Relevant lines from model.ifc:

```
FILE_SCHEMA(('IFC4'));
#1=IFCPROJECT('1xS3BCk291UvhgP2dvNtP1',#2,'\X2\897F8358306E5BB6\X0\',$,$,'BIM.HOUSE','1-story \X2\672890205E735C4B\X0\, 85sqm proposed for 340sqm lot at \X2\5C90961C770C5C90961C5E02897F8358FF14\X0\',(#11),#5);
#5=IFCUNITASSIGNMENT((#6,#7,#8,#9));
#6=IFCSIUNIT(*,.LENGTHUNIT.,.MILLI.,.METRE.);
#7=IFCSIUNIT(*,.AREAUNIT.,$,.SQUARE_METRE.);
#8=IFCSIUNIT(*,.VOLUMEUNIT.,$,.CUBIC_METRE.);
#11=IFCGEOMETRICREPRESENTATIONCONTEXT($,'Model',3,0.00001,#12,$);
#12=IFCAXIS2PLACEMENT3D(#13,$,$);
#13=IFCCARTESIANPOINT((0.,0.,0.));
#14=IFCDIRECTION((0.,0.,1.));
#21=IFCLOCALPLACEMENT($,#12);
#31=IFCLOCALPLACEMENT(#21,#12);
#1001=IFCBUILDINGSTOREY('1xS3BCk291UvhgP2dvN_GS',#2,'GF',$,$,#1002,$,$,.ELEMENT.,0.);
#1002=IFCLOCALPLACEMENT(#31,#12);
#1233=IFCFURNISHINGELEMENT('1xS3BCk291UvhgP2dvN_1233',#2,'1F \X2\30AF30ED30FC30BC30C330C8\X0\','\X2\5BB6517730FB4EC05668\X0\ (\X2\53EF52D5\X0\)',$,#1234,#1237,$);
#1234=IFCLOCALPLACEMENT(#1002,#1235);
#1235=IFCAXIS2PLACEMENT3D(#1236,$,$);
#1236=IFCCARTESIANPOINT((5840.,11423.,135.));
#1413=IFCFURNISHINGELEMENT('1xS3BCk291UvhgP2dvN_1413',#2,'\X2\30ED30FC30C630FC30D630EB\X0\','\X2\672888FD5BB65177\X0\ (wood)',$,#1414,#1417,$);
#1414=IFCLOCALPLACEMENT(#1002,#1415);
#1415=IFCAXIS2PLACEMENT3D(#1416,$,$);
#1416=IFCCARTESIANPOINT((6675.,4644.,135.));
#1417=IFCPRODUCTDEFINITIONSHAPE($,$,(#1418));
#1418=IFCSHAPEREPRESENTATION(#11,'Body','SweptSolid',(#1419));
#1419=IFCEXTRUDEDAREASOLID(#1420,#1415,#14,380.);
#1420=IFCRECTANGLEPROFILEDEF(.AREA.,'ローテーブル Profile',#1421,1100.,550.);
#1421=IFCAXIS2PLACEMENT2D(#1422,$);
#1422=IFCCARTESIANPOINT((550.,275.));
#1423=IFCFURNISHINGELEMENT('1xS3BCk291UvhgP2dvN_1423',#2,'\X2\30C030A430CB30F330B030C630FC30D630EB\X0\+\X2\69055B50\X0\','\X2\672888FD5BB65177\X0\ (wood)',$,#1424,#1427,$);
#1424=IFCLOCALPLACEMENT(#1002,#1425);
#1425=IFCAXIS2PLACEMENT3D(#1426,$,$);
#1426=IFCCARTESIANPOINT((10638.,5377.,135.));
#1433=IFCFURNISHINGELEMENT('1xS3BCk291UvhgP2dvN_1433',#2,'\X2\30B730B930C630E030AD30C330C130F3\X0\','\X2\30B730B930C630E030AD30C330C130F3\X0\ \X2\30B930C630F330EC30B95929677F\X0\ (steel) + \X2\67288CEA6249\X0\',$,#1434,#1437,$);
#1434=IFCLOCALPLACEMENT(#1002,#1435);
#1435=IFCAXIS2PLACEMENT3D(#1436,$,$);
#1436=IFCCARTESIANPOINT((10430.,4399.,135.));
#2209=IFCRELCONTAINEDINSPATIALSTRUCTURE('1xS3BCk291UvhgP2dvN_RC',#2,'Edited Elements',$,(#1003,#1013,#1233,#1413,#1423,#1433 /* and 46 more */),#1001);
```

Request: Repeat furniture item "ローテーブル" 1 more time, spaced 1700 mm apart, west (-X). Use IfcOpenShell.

```python
import numpy as np
import ifcopenshell
import ifcopenshell.api.geometry
import ifcopenshell.api.root
import ifcopenshell.util.element
import ifcopenshell.util.placement
import ifcopenshell.util.unit

model = ifcopenshell.open("model.ifc")
unit_scale = ifcopenshell.util.unit.calculate_unit_scale(model)


def reuse_history(source, copy):
    """copy_class also copies each property set's owner history, people and application; keep the originals."""
    for rel in copy.IsDefinedBy:
        if rel.is_a("IfcRelDefinesByProperties") and (history := rel.RelatingPropertyDefinition.OwnerHistory):
            rel.RelatingPropertyDefinition.OwnerHistory = source.OwnerHistory
            ifcopenshell.util.element.remove_deep2(model, history)


source = model.by_guid("1xS3BCk291UvhgP2dvN_1413")
base = ifcopenshell.util.placement.get_local_placement(source.ObjectPlacement)
step = np.array([-1.0, 0.0, 0.0]) * 1.7 / unit_scale

for i in range(1, 2):
    copy = ifcopenshell.api.root.copy_class(model, product=source)
    copy.Representation = ifcopenshell.util.element.copy_deep(
        model, source.Representation, exclude=["IfcGeometricRepresentationContext", "IfcRepresentationMap"]
    )
    reuse_history(source, copy)
    matrix = base.copy()
    matrix[:3, 3] += i * step
    print("added at", matrix[:3, 3].round(3) + 0.0)
    ifcopenshell.api.geometry.edit_object_placement(model, product=copy, matrix=matrix, is_si=False)

model.write("model_rev.ifc")
```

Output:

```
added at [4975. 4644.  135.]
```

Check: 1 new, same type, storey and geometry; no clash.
